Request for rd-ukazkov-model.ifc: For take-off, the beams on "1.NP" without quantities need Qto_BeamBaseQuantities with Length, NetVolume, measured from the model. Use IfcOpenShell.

First a look at what the model holds.

```python
import ifcopenshell
import ifcopenshell.util.element
import ifcopenshell.util.unit

model = ifcopenshell.open("rd-ukazkov-model.ifc")
print(model.schema)
for unit_type in ("LENGTHUNIT", "AREAUNIT", "VOLUMEUNIT"):
    print(unit_type, ifcopenshell.util.unit.calculate_unit_scale(model, unit_type))
storey = next(s for s in model.by_type("IfcBuildingStorey") if s.Name == "1.NP")
beams = [e for e in ifcopenshell.util.element.get_decomposition(storey) if e.is_a("IfcBeam")]
for e in sorted(beams, key=lambda e: e.id()):
    print(e.id(), e.is_a(), e.Name, list(ifcopenshell.util.element.get_psets(e, qtos_only=True)), sep=" | ")
```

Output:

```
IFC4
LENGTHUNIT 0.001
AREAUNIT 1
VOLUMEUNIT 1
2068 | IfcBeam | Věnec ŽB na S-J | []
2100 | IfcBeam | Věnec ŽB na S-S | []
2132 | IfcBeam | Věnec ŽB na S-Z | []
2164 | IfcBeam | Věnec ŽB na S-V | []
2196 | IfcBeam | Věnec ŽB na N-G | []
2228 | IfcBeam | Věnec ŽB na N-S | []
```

```python
import ifcopenshell
import ifcopenshell.api.pset
import ifcopenshell.geom
import ifcopenshell.util.element
import ifcopenshell.util.shape
import ifcopenshell.util.unit

model = ifcopenshell.open("rd-ukazkov-model.ifc")
unit_scale = ifcopenshell.util.unit.calculate_unit_scale(model)
volume_scale = ifcopenshell.util.unit.calculate_unit_scale(model, "VOLUMEUNIT")
settings = ifcopenshell.geom.settings()

storey = next(s for s in model.by_type("IfcBuildingStorey") if s.Name == "1.NP")
beams = [e for e in ifcopenshell.util.element.get_decomposition(storey) if e.is_a("IfcBeam")]

for e in sorted(beams, key=lambda e: e.id()):
    if ifcopenshell.util.element.get_psets(e, qtos_only=True, should_inherit=False):
        continue
    # Geometry comes back in metres, in the element's own axes.
    shape = ifcopenshell.geom.create_shape(settings, e)
    values = {
        "Length": ifcopenshell.util.shape.get_max_xyz(shape.geometry) / unit_scale,
        "NetVolume": ifcopenshell.util.shape.get_volume(shape.geometry) / volume_scale,
    }
    qto = ifcopenshell.api.pset.add_qto(model, product=e, name="Qto_BeamBaseQuantities")
    ifcopenshell.api.pset.edit_qto(model, qto=qto, properties=values)
    print(e.id(), {k: round(v, 3) for k, v in values.items()})

model.write("rd-ukazkov-model_v2.ifc")
```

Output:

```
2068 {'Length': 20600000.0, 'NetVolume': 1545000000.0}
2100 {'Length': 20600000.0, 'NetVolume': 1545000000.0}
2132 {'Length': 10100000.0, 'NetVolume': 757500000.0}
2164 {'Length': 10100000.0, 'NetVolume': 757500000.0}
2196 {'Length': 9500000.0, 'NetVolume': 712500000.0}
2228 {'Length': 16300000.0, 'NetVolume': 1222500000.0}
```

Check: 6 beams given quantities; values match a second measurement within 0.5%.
